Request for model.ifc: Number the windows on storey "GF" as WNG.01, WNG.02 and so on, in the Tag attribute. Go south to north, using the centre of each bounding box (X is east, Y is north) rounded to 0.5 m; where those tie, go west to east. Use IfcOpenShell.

First a look at what the model holds.

```python
import ifcopenshell
import ifcopenshell.util.element
import ifcopenshell.util.placement

model = ifcopenshell.open("model.ifc")
print(model.schema)
storey = next(s for s in model.by_type("IfcBuildingStorey") if s.Name == "GF")
windows = [e for e in ifcopenshell.util.element.get_decomposition(storey) if e.is_a("IfcWindow")]
for e in sorted(windows, key=lambda e: e.id()):
    origin = ifcopenshell.util.placement.get_local_placement(e.ObjectPlacement)[:3, 3]
    print(e.id(), e.Tag, e.Name, origin.round(2) + 0.0, sep=" | ")
```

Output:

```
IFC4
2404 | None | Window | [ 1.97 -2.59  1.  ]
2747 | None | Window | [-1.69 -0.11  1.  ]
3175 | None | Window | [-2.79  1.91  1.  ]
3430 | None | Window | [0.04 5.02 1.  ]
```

```python
import ifcopenshell
import ifcopenshell.geom
import ifcopenshell.util.element
import ifcopenshell.util.shape

model = ifcopenshell.open("model.ifc")
settings = ifcopenshell.geom.settings()
settings.set("use-world-coords", True)


def centre(element):
    shape = ifcopenshell.geom.create_shape(settings, element)
    return ifcopenshell.util.shape.get_bbox_centroid(shape.geometry)


storey = next(s for s in model.by_type("IfcBuildingStorey") if s.Name == "GF")
windows = [e for e in ifcopenshell.util.element.get_decomposition(storey) if e.is_a("IfcWindow")]

# Insertion points can sit at a corner or the storey origin, so sort by the geometry (in metres).
centres = {e: centre(e) for e in windows}
windows.sort(key=lambda e: (round(centres[e][1] / 0.5), centres[e][0]))

for i, e in enumerate(windows, start=1):
    number = f"WNG.{i:02d}"
    e.Tag = number
    print(e.id(), number)

model.write("model-out.ifc")
```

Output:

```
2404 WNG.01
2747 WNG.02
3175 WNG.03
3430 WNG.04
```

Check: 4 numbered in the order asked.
